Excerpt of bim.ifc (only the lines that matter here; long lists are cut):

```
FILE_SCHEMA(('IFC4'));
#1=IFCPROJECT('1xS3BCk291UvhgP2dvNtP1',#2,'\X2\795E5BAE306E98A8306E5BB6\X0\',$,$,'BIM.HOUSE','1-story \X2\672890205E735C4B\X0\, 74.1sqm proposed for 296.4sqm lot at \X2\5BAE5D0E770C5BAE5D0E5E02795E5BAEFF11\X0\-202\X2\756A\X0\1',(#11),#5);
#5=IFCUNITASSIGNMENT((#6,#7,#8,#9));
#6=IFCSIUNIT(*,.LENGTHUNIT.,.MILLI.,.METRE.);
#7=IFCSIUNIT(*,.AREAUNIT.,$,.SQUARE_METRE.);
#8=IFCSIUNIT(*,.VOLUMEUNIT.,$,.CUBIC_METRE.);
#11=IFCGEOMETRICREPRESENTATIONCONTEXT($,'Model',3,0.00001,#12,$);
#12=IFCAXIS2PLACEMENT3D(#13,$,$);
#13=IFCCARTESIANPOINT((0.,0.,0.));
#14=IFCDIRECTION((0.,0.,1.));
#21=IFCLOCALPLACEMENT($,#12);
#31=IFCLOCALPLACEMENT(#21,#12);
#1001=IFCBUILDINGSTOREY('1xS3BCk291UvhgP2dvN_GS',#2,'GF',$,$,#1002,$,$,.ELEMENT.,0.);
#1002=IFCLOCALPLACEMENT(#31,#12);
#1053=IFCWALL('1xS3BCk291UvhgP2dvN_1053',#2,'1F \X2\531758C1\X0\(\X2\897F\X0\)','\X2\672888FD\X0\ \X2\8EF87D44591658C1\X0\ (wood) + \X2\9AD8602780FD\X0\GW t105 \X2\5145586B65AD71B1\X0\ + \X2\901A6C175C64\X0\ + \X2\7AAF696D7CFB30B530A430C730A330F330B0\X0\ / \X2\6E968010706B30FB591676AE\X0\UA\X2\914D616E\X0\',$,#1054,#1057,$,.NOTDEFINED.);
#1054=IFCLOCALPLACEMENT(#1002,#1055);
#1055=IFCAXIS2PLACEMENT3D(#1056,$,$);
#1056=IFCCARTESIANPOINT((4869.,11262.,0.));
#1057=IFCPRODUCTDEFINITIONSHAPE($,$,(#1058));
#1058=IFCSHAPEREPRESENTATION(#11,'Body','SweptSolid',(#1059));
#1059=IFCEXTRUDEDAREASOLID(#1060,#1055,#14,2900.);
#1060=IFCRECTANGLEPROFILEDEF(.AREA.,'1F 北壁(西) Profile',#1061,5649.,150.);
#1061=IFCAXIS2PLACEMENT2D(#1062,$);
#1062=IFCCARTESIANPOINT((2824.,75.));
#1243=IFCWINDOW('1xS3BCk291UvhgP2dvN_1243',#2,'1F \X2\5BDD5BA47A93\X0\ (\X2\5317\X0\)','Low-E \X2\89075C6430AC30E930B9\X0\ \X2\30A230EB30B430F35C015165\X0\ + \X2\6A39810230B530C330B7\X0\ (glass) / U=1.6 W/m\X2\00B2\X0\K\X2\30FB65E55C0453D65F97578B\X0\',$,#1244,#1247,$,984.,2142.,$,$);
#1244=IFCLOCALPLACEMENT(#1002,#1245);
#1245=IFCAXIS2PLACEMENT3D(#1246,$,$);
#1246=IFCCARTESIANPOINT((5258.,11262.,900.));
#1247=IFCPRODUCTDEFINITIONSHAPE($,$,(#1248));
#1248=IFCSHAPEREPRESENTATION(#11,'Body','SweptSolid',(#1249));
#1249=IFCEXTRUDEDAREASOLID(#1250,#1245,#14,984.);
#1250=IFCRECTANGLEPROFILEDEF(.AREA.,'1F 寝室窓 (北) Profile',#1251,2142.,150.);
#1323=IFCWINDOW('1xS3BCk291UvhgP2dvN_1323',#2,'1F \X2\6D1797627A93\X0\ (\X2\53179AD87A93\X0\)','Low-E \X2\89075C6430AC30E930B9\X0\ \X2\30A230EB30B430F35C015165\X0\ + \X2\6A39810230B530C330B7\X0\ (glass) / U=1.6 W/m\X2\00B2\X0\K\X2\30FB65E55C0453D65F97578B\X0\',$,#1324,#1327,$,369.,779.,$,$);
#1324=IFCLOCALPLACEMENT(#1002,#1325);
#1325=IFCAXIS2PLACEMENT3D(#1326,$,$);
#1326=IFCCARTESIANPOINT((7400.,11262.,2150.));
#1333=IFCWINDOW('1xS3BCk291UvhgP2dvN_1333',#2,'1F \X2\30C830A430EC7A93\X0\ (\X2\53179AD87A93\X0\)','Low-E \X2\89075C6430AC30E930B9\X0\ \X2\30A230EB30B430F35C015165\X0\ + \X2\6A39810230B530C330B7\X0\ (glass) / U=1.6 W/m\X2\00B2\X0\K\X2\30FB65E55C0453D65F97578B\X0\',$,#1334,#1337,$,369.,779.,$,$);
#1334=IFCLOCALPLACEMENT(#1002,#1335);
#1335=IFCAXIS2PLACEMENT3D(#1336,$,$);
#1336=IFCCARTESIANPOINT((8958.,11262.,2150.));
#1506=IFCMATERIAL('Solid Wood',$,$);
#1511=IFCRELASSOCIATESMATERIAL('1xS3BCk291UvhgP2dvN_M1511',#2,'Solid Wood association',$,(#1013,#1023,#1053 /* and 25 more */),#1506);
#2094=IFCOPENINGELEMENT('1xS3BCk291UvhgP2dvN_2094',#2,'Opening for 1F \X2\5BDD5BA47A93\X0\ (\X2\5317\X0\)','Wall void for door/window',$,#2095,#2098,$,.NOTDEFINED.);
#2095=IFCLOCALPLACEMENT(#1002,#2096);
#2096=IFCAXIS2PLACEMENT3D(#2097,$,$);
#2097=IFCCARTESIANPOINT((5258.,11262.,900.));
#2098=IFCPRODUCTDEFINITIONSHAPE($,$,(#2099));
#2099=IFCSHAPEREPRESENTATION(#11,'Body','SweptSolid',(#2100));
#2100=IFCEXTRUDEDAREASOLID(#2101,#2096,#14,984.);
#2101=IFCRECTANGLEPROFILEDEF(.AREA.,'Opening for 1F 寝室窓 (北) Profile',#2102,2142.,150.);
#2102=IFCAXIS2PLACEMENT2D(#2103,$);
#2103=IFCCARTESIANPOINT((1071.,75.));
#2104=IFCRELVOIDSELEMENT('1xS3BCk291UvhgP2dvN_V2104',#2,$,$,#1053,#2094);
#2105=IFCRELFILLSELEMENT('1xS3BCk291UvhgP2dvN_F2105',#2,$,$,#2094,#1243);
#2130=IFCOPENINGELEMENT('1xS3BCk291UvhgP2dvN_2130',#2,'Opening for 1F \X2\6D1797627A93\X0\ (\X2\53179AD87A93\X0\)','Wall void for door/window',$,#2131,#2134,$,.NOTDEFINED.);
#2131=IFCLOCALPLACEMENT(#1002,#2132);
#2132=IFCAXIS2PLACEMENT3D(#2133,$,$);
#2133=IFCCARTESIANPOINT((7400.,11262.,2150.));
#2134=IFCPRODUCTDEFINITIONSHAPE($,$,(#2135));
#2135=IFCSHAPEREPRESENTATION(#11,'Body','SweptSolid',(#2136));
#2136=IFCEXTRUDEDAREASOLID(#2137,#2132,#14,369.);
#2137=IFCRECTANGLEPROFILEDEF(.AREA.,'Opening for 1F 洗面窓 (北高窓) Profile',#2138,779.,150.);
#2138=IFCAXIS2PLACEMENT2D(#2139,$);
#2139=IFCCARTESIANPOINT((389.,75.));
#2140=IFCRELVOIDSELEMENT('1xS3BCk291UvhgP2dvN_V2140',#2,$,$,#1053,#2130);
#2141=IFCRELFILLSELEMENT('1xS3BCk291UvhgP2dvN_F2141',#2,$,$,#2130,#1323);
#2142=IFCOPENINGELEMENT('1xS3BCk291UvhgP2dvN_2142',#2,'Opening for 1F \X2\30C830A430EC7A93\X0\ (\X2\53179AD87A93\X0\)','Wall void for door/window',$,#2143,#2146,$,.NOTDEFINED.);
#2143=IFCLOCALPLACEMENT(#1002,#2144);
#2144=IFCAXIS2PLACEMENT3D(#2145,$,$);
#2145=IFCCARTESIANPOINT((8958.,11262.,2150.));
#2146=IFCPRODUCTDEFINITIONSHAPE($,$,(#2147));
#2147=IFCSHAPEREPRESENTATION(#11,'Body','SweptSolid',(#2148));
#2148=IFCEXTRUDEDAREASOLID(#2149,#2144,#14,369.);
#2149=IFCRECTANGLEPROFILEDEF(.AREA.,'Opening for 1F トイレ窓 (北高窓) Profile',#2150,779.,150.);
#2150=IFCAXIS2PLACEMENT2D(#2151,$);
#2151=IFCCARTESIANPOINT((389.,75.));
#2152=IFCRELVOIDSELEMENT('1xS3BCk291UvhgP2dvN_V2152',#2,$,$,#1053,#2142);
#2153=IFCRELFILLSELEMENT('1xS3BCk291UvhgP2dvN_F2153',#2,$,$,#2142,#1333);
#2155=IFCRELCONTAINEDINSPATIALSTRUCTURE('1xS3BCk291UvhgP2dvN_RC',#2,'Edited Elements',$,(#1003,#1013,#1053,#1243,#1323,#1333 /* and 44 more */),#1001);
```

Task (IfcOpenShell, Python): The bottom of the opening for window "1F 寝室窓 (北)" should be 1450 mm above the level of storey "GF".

```python
import numpy as np
import ifcopenshell
import ifcopenshell.api.geometry
import ifcopenshell.geom
import ifcopenshell.util.element
import ifcopenshell.util.placement
import ifcopenshell.util.shape
import ifcopenshell.util.unit

model = ifcopenshell.open("bim.ifc")
unit_scale = ifcopenshell.util.unit.calculate_unit_scale(model)

window = model.by_id(1243)
opening = window.FillsVoids[0].RelatingOpeningElement
storey = ifcopenshell.util.element.get_container(window, ifc_class="IfcBuildingStorey")
level = ifcopenshell.util.placement.get_local_placement(storey.ObjectPlacement)[2, 3]

# The opening's origin need not be at the sill, so measure its lowest point.
shape = ifcopenshell.geom.create_shape(ifcopenshell.geom.settings(), opening)
bottom = ifcopenshell.util.shape.get_shape_bottom_elevation(shape, shape.geometry) / unit_scale
dz = level + 1.45 / unit_scale - bottom

shift = np.array([0.0, 0.0, dz])
# The window is not placed relative to its opening, so move both.
for product in (opening, window):
    matrix = ifcopenshell.util.placement.get_local_placement(product.ObjectPlacement)
    matrix[:3, 3] += shift
    ifcopenshell.api.geometry.edit_object_placement(model, product=product, matrix=matrix, is_si=False)

print(f"moved by {dz * unit_scale:+.3f} m")

model.write("bim_rev.ifc")
```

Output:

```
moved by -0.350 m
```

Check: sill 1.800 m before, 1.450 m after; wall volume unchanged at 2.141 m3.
